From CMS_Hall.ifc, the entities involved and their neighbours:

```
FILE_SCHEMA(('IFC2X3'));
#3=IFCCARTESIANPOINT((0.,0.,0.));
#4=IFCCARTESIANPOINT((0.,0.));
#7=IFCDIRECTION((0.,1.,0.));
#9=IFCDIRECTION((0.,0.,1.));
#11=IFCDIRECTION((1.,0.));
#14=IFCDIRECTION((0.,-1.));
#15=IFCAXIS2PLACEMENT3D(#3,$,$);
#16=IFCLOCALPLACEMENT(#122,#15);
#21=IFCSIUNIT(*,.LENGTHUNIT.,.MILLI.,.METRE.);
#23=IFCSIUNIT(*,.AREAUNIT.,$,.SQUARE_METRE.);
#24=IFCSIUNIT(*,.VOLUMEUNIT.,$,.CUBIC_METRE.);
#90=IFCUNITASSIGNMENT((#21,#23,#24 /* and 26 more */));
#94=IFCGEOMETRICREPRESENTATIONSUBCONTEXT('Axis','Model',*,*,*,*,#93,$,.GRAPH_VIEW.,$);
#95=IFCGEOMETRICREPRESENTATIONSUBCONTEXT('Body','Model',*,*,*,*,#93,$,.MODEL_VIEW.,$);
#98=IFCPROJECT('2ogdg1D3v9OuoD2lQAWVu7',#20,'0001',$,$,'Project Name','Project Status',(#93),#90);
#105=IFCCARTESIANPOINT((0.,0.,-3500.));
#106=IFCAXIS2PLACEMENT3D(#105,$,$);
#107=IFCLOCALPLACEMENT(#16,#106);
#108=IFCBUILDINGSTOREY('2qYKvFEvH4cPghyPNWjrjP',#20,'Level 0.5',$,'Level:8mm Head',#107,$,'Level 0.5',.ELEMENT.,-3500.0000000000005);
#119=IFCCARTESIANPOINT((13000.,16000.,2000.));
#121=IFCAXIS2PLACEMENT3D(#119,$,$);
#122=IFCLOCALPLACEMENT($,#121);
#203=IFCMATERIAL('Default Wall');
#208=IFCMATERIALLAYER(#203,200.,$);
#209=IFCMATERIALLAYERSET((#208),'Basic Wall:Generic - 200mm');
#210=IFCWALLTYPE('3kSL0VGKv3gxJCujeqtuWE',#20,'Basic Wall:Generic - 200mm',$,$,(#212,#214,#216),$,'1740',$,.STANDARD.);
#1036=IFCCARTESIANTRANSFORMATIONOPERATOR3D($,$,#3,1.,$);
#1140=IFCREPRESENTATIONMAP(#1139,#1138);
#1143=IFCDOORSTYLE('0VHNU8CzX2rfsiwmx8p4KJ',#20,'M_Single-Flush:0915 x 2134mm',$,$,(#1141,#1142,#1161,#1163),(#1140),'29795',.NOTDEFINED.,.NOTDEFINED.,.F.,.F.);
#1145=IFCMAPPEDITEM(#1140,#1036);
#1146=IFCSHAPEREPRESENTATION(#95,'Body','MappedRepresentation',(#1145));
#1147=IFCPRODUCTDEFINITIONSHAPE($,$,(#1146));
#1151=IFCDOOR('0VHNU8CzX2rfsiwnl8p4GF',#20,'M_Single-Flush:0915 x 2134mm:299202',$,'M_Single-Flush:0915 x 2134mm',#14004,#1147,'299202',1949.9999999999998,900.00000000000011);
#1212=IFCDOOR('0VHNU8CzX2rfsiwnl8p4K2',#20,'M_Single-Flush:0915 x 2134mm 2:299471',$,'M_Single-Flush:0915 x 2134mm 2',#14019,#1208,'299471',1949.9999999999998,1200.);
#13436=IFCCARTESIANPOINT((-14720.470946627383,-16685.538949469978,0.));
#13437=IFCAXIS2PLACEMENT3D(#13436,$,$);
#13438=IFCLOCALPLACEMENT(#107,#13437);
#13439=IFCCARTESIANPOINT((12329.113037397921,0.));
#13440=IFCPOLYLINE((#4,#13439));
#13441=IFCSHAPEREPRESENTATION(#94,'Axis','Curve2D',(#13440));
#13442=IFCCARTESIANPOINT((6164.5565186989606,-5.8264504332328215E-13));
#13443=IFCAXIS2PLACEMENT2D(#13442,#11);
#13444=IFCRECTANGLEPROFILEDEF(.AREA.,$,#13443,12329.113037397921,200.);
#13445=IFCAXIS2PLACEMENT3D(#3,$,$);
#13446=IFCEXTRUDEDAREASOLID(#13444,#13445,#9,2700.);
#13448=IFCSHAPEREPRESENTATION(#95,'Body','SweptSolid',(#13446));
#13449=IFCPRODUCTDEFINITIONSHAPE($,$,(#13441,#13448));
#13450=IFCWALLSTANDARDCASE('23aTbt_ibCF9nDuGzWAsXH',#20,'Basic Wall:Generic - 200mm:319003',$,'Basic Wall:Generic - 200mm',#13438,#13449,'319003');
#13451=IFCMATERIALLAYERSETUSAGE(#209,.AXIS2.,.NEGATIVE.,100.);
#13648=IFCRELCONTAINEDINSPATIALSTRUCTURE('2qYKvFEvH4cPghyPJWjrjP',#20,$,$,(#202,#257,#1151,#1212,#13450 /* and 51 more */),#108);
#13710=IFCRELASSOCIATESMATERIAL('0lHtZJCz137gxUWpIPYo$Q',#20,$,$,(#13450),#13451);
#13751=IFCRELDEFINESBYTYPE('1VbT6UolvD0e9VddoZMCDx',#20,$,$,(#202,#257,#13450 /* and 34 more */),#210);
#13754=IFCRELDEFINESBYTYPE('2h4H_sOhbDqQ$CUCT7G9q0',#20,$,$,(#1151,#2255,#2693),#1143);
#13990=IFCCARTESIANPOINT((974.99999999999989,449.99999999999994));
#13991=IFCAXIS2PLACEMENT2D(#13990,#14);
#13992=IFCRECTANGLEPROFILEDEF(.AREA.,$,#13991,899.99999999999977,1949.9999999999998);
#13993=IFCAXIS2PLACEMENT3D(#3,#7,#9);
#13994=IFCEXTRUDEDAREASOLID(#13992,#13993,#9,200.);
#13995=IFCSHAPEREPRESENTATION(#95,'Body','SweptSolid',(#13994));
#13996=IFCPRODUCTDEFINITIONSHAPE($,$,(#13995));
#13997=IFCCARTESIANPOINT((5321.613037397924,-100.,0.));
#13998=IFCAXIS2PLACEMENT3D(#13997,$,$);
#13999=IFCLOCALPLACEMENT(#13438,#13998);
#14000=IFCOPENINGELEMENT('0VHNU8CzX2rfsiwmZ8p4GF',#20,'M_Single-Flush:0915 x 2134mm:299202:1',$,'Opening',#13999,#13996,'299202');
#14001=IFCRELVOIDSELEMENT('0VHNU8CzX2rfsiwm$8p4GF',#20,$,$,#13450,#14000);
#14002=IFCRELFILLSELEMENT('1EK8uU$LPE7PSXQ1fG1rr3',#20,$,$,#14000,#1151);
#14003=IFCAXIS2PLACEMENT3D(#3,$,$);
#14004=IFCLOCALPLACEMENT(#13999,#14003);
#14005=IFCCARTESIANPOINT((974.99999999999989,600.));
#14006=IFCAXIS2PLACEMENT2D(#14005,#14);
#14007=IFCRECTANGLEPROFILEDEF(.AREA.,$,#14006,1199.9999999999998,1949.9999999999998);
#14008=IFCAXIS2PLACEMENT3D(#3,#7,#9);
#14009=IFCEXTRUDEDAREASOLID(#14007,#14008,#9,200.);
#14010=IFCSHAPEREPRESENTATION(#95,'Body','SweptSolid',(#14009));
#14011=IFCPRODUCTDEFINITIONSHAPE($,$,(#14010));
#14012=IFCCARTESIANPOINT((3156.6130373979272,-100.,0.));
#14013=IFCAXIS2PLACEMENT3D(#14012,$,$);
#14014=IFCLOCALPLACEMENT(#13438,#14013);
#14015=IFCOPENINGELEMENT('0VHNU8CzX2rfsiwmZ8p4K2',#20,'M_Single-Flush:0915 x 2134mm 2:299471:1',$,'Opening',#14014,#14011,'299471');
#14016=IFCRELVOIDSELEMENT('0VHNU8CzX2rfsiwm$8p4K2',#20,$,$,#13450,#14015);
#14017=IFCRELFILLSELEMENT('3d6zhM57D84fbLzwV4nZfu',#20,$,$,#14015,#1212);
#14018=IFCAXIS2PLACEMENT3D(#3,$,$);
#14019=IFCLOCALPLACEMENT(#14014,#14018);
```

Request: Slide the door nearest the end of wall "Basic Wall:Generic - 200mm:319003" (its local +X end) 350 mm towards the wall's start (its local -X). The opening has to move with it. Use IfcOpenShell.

```python
import ifcopenshell
import ifcopenshell.api.geometry
import ifcopenshell.util.placement

model = ifcopenshell.open("CMS_Hall.ifc")

door = model.by_guid("0VHNU8CzX2rfsiwnl8p4GF")
opening = door.FillsVoids[0].RelatingOpeningElement
wall = opening.VoidsElements[0].RelatingBuildingElement

wall_matrix = ifcopenshell.util.placement.get_local_placement(wall.ObjectPlacement)
shift = wall_matrix[:3, 0] * -350.0
before = ifcopenshell.util.placement.get_local_placement(door.ObjectPlacement)[:3, 3].copy()

# The door is placed relative to its opening, so it follows when the opening moves.
matrix = ifcopenshell.util.placement.get_local_placement(opening.ObjectPlacement)
matrix[:3, 3] += shift
ifcopenshell.api.geometry.edit_object_placement(
    model, product=opening, matrix=matrix, is_si=False, should_transform_children=True
)

after = ifcopenshell.util.placement.get_local_placement(door.ObjectPlacement)[:3, 3]
print("door moved by", (after - before).round(3) + 0.0)

model.write("CMS_Hall_v2.ifc")
```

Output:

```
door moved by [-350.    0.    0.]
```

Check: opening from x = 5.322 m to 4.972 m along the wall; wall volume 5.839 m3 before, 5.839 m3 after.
